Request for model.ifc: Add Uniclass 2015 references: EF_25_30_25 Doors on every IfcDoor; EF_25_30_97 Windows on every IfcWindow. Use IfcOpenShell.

First a look at what the model holds.

```python
import ifcopenshell

model = ifcopenshell.open("model.ifc")
print(model.schema)
print("classifications:", [c.Name for c in model.by_type("IfcClassification")])
for ifc_class in ("IfcDoor", "IfcRoof", "IfcStair", "IfcWall", "IfcWindow"):
    print(ifc_class, len(model.by_type(ifc_class)))
```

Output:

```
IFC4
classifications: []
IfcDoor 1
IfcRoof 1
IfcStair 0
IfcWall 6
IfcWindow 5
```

```python
import ifcopenshell
import ifcopenshell.api.classification

model = ifcopenshell.open("model.ifc")

system = ifcopenshell.api.classification.add_classification(model, classification="Uniclass 2015")

codes = {
    "IfcDoor": ("EF_25_30_25", "Doors"),
    "IfcWindow": ("EF_25_30_97", "Windows"),
}
for ifc_class, (code, name) in codes.items():
    products = model.by_type(ifc_class)
    ifcopenshell.api.classification.add_reference(
        model, products=products, classification=system, identification=code, name=name
    )
    print(code, len(products))

model.write("model_edited.ifc")
```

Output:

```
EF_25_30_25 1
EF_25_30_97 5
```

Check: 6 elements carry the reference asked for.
